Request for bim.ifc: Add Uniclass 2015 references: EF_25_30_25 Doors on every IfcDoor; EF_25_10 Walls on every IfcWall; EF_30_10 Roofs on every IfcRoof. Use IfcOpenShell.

First a look at what the model holds.

```python
import ifcopenshell

model = ifcopenshell.open("bim.ifc")
print(model.schema)
print("classifications:", [c.Name for c in model.by_type("IfcClassification")])
for ifc_class in ("IfcDoor", "IfcRoof", "IfcStair", "IfcWall", "IfcWindow"):
    print(ifc_class, len(model.by_type(ifc_class)))
```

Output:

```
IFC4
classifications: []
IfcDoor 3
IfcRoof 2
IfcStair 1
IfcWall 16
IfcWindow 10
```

```python
import ifcopenshell
import ifcopenshell.api.classification

model = ifcopenshell.open("bim.ifc")

system = ifcopenshell.api.classification.add_classification(model, classification="Uniclass 2015")

codes = {
    "IfcDoor": ("EF_25_30_25", "Doors"),
    "IfcWall": ("EF_25_10", "Walls"),
    "IfcRoof": ("EF_30_10", "Roofs"),
}
for ifc_class, (code, name) in codes.items():
    products = model.by_type(ifc_class)
    ifcopenshell.api.classification.add_reference(
        model, products=products, classification=system, identification=code, name=name
    )
    print(code, len(products))

model.write("bim-out.ifc")
```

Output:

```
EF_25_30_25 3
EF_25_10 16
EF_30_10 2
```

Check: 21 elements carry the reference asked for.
